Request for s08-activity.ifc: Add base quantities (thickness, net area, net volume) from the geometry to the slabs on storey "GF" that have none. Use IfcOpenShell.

First a look at what the model holds.

```python
import ifcopenshell
import ifcopenshell.util.element
import ifcopenshell.util.unit

model = ifcopenshell.open("s08-activity.ifc")
print(model.schema)
for unit_type in ("LENGTHUNIT", "AREAUNIT", "VOLUMEUNIT"):
    print(unit_type, ifcopenshell.util.unit.calculate_unit_scale(model, unit_type))
storey = next(s for s in model.by_type("IfcBuildingStorey") if s.Name == "GF")
slabs = [e for e in ifcopenshell.util.element.get_decomposition(storey) if e.is_a("IfcSlab")]
for e in sorted(slabs, key=lambda e: e.id()):
    print(e.id(), e.is_a(), e.Name, list(ifcopenshell.util.element.get_psets(e, qtos_only=True)), sep=" | ")
```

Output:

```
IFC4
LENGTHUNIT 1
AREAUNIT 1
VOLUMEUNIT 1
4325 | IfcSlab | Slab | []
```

```python
import ifcopenshell
import ifcopenshell.api.pset
import ifcopenshell.geom
import ifcopenshell.util.element
import ifcopenshell.util.shape
import ifcopenshell.util.unit

model = ifcopenshell.open("s08-activity.ifc")
unit_scale = ifcopenshell.util.unit.calculate_unit_scale(model)
area_scale = ifcopenshell.util.unit.calculate_unit_scale(model, "AREAUNIT")
volume_scale = ifcopenshell.util.unit.calculate_unit_scale(model, "VOLUMEUNIT")
settings = ifcopenshell.geom.settings()

storey = next(s for s in model.by_type("IfcBuildingStorey") if s.Name == "GF")
slabs = [e for e in ifcopenshell.util.element.get_decomposition(storey) if e.is_a("IfcSlab")]

for e in sorted(slabs, key=lambda e: e.id()):
    if ifcopenshell.util.element.get_psets(e, qtos_only=True, should_inherit=False):
        continue
    # Geometry comes back in metres, in the element's own axes.
    shape = ifcopenshell.geom.create_shape(settings, e)
    values = {
        "Width": ifcopenshell.util.shape.get_z(shape.geometry) / unit_scale,
        "NetArea": ifcopenshell.util.shape.get_footprint_area(shape.geometry) / area_scale,
        "NetVolume": ifcopenshell.util.shape.get_volume(shape.geometry) / volume_scale,
    }
    qto = ifcopenshell.api.pset.add_qto(model, product=e, name="Qto_SlabBaseQuantities")
    ifcopenshell.api.pset.edit_qto(model, qto=qto, properties=values)
    print(e.id(), {k: round(v, 3) for k, v in values.items()})

model.write("s08-activity_edited.ifc")
```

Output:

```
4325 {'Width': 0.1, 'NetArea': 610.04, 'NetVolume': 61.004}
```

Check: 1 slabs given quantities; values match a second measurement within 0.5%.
